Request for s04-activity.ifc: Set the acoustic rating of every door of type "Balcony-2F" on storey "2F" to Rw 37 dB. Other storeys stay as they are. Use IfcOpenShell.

First a look at what the model holds.

```python
import ifcopenshell
import ifcopenshell.util.element

model = ifcopenshell.open("s04-activity.ifc")
print(model.schema)
storey = next(s for s in model.by_type("IfcBuildingStorey") if s.Name == "2F")
doors = [e for e in ifcopenshell.util.element.get_decomposition(storey) if e.is_a("IfcDoor")]
seen = {}
for e in doors:
    element_type = ifcopenshell.util.element.get_type(e)
    key = (element_type.Name if element_type != e and element_type else None, ifcopenshell.util.element.get_pset(e, "Pset_DoorCommon", "AcousticRating"))
    seen[key] = seen.get(key, 0) + 1
for (name, value), count in sorted(seen.items(), key=str):
    print(count, "x", name, "|", value)
```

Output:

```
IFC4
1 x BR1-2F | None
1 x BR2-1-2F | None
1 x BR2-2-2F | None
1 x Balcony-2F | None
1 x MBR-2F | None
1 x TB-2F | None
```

```python
import ifcopenshell
import ifcopenshell.api.pset
import ifcopenshell.util.element

model = ifcopenshell.open("s04-activity.ifc")

storey = next(s for s in model.by_type("IfcBuildingStorey") if s.Name == "2F")
doors = [e for e in ifcopenshell.util.element.get_decomposition(storey) if e.is_a("IfcDoor")]

count = 0
for e in doors:
    element_type = ifcopenshell.util.element.get_type(e)
    if element_type in (None, e) or element_type.Name != "Balcony-2F":
        continue
    # add_pset returns the element's existing set when there is one.
    pset = ifcopenshell.api.pset.add_pset(model, product=e, name="Pset_DoorCommon")
    ifcopenshell.api.pset.edit_pset(model, pset=pset, properties={"AcousticRating": "Rw 37 dB"})
    count += 1

print(count, "doors updated")

model.write("s04-activity_v2.ifc")
```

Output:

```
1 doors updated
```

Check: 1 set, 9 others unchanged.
